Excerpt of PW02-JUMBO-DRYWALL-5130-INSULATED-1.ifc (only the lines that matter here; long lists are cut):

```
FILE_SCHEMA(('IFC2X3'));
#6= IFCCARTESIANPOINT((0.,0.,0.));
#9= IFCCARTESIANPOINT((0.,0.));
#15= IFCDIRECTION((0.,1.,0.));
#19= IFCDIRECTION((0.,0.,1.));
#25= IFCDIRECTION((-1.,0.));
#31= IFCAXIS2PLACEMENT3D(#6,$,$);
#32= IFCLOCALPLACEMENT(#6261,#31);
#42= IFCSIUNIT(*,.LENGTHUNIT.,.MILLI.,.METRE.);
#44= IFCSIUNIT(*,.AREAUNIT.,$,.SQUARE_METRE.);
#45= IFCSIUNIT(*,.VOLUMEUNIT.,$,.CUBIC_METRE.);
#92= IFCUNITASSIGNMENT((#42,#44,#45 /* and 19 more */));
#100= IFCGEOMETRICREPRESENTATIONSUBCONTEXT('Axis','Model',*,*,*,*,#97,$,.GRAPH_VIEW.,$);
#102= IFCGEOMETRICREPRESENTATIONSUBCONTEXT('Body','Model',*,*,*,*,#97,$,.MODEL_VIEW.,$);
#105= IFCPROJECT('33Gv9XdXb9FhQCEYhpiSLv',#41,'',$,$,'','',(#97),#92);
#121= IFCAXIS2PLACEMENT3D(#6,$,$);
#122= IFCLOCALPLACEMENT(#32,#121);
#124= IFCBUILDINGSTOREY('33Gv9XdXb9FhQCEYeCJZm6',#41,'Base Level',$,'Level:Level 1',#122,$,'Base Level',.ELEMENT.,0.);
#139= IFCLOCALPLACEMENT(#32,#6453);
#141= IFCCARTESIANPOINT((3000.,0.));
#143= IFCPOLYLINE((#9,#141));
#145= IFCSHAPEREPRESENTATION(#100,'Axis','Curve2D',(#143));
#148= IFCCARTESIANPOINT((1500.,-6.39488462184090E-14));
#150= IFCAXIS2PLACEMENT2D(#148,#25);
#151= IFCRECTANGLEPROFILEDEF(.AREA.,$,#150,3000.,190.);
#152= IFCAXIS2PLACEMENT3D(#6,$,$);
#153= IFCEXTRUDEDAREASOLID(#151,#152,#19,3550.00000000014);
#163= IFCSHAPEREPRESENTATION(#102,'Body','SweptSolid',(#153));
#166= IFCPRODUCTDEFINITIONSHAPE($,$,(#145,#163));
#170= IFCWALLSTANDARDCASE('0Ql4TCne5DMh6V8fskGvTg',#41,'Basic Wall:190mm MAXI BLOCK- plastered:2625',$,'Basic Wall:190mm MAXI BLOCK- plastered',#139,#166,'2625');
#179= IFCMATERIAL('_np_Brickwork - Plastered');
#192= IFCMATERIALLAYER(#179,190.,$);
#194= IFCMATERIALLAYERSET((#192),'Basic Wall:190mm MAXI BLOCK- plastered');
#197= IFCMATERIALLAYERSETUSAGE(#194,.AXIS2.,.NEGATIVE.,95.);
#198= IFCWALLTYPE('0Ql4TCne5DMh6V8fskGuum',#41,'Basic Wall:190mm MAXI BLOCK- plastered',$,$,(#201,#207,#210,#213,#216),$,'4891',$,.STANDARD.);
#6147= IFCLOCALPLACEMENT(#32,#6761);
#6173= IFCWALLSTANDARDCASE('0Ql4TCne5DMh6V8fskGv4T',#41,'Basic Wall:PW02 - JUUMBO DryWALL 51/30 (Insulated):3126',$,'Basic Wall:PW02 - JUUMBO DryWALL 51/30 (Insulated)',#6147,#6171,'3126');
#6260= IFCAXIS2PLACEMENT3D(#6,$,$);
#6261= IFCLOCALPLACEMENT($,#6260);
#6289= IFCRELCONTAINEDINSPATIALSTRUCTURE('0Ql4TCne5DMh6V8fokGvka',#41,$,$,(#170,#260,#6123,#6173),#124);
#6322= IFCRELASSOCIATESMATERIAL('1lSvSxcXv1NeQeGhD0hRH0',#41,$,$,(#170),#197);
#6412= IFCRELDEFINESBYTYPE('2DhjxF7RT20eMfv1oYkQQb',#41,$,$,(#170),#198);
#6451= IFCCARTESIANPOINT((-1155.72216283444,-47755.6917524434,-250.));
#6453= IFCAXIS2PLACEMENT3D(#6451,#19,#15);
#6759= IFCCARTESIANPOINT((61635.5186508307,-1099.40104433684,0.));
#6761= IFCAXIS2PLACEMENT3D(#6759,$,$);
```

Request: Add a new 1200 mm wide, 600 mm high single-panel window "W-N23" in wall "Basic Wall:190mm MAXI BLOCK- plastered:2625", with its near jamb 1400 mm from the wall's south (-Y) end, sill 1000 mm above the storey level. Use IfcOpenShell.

```python
import numpy as np
import ifcopenshell
import ifcopenshell.api.feature
import ifcopenshell.api.geometry
import ifcopenshell.api.root
import ifcopenshell.api.spatial
import ifcopenshell.api.type
import ifcopenshell.geom
import ifcopenshell.util.element
import ifcopenshell.util.placement
import ifcopenshell.util.representation
import ifcopenshell.util.shape
import ifcopenshell.util.unit

model = ifcopenshell.open("PW02-JUMBO-DRYWALL-5130-INSULATED-1.ifc")
unit_scale = ifcopenshell.util.unit.calculate_unit_scale(model)
settings = ifcopenshell.geom.settings()


def volume(element):
    """Net volume in cubic metres, openings subtracted."""
    shape = ifcopenshell.geom.create_shape(settings, element)
    return ifcopenshell.util.shape.get_volume(shape.geometry)


wall = model.by_guid("0Ql4TCne5DMh6V8fskGvTg")
storey = ifcopenshell.util.element.get_container(wall, ifc_class="IfcBuildingStorey")
context = ifcopenshell.util.representation.get_context(model, "Model", "Body", "MODEL_VIEW")
before = volume(wall)

width, height, from_end, sill = 1.2, 0.6, 1.4, 1  # metres

# The wall runs along its own X axis, and the end named is its -X end.
wall_shape = ifcopenshell.geom.create_shape(settings, wall)
x, y, z = ifcopenshell.util.shape.get_vertices(wall_shape.geometry).T
start = x.min() + from_end
face, thickness = float(y.min()), float(y.max() - y.min())
wall_matrix = ifcopenshell.util.placement.get_local_placement(wall.ObjectPlacement)
level = ifcopenshell.util.placement.get_local_placement(storey.ObjectPlacement)[2, 3]


def in_wall(x, y):
    """Placement at x, y metres in the wall's axes, at sill height."""
    matrix = wall_matrix.copy()
    matrix[:, 3] = wall_matrix @ np.array([x / unit_scale, y / unit_scale, 0.0, 1.0])
    matrix[2, 3] = level + sill / unit_scale
    return matrix


# Opening: a box that overshoots both wall faces by 50 mm.
opening = ifcopenshell.api.root.create_entity(model, ifc_class="IfcOpeningElement")
box = ifcopenshell.api.geometry.add_wall_representation(
    model, context=context, length=width, height=height, thickness=thickness + 0.1
)
ifcopenshell.api.geometry.assign_representation(model, product=opening, representation=box)
ifcopenshell.api.geometry.edit_object_placement(model, product=opening, matrix=in_wall(start, face - 0.05), is_si=False)
ifcopenshell.api.feature.add_feature(model, feature=opening, element=wall)

window = ifcopenshell.api.root.create_entity(model, ifc_class="IfcWindow", name="W-N23")
window.OverallWidth, window.OverallHeight = width / unit_scale, height / unit_scale
body = ifcopenshell.api.geometry.add_window_representation(
    model,
    context=context,
    overall_width=window.OverallWidth,
    overall_height=window.OverallHeight,
    partition_type="SINGLE_PANEL",
)
ifcopenshell.api.geometry.assign_representation(model, product=window, representation=body)
ifcopenshell.api.spatial.assign_container(model, products=[window], relating_structure=storey)
fills = ifcopenshell.api.feature.add_filling(model, opening=opening, element=window)
fills.OwnerHistory = window.OwnerHistory  # required in IFC2X3

# IFC2X3 keeps the operation on the window style.
style = ifcopenshell.api.root.create_entity(model, ifc_class="IfcWindowStyle", name="W-N23")
style.OperationType, style.ConstructionType = "SINGLE_PANEL", "NOTDEFINED"
style.ParameterTakesPrecedence = style.Sizeable = False
ifcopenshell.api.type.assign_type(model, related_objects=[window], relating_type=style)

# Centre the window in the wall's thickness.
ifcopenshell.api.geometry.edit_object_placement(model, product=window, matrix=in_wall(start, face), is_si=False)
window_shape = ifcopenshell.geom.create_shape(settings, window)
depth = ifcopenshell.util.shape.get_vertices(window_shape.geometry)[:, 1]
offset = face + thickness / 2 - (depth.min() + depth.max()) / 2
ifcopenshell.api.geometry.edit_object_placement(model, product=window, matrix=in_wall(start, offset), is_si=False)

after = volume(wall)

print(f"wall volume {before:.3f} -> {after:.3f} m3")

model.write("PW02-JUMBO-DRYWALL-5130-INSULATED-1_edited.ifc")
```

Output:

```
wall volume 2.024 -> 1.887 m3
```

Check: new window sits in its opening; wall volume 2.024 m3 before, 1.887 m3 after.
